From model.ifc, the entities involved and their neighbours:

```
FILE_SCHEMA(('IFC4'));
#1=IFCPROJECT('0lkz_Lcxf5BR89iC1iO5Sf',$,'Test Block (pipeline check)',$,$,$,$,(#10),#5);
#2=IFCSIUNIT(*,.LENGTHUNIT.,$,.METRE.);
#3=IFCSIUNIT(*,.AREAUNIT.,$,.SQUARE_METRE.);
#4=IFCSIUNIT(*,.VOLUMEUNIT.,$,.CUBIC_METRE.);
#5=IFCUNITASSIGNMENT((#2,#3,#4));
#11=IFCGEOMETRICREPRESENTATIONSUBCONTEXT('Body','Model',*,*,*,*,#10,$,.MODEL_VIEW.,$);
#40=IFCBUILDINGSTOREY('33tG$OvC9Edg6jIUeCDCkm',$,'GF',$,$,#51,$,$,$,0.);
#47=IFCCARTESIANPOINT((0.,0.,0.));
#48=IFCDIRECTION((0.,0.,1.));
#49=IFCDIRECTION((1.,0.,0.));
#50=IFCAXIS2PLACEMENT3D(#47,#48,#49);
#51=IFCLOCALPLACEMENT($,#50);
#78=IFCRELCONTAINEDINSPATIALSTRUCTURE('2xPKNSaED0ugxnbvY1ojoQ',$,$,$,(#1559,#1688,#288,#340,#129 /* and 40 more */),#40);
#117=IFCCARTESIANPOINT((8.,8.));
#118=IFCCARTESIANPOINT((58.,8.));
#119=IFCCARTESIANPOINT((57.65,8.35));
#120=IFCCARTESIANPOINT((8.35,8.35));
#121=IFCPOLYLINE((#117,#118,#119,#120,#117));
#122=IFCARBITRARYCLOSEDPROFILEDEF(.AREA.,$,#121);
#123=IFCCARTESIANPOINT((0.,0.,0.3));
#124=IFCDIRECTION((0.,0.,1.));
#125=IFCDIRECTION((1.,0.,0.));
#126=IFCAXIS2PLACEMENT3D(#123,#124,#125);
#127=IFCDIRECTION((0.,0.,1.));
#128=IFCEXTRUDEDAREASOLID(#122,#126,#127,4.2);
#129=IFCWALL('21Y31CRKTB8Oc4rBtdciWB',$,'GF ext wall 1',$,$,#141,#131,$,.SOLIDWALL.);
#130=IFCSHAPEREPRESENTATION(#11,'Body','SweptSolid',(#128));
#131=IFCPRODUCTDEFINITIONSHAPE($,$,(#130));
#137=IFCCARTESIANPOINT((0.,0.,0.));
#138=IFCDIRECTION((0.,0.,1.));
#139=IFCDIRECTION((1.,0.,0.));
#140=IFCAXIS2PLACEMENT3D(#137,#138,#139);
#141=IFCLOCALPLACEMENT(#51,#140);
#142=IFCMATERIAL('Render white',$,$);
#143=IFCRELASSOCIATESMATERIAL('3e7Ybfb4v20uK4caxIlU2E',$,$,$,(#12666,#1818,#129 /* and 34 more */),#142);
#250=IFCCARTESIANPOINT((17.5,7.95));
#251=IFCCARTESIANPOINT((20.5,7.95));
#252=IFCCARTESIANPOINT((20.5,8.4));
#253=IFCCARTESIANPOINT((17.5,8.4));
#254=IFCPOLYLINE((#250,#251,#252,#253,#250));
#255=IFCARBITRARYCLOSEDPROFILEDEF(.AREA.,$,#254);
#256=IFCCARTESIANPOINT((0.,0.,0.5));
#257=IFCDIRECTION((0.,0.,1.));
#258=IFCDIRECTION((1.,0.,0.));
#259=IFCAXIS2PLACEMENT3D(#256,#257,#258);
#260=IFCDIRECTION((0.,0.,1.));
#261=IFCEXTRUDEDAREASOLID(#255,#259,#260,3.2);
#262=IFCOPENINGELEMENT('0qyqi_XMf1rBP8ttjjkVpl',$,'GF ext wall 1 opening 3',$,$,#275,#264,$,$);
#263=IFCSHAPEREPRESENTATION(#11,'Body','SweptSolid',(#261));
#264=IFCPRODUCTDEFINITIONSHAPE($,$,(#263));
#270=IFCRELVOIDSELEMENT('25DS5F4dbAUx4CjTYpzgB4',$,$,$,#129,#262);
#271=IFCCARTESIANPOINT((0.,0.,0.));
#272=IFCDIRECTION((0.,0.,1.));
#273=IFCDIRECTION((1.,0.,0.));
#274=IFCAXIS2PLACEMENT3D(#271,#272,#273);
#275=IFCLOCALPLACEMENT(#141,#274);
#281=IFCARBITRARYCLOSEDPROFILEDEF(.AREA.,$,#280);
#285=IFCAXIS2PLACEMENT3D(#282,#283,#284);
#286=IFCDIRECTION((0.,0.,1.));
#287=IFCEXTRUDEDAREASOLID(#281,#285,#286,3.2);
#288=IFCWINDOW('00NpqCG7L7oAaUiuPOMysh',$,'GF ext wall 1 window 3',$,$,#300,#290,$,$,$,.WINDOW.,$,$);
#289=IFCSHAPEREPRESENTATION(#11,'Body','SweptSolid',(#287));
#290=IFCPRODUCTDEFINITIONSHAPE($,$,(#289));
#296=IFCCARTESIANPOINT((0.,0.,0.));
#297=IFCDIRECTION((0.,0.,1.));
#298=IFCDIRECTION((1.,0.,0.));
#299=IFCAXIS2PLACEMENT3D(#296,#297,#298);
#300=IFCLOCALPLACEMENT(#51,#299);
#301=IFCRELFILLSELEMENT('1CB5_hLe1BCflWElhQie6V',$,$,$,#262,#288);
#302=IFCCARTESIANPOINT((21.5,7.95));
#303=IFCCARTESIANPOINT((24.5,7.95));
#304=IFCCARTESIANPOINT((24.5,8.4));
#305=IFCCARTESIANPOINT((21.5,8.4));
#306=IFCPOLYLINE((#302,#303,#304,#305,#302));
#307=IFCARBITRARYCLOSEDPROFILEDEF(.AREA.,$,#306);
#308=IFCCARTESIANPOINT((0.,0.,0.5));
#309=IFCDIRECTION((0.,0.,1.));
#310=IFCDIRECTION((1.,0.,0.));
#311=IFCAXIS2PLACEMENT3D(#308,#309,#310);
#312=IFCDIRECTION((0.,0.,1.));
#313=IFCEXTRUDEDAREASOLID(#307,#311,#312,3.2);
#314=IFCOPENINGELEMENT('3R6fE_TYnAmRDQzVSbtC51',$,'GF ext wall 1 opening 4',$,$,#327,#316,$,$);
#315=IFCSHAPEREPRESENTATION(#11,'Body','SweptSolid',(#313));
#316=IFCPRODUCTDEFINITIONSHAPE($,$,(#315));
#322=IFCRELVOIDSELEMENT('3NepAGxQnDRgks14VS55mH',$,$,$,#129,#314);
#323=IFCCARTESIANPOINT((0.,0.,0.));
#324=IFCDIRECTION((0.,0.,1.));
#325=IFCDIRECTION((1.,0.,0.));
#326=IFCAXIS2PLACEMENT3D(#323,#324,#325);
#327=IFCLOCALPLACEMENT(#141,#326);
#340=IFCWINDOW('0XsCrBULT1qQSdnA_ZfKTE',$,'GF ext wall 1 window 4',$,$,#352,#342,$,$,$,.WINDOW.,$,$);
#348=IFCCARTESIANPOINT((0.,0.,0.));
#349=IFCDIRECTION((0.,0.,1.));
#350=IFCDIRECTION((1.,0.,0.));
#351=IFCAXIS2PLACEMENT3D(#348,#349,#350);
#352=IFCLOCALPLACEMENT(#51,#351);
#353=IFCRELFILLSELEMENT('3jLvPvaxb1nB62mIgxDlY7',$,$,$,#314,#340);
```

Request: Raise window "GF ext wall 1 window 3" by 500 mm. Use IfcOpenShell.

```python
import numpy as np
import ifcopenshell
import ifcopenshell.api.geometry
import ifcopenshell.util.placement
import ifcopenshell.util.unit

model = ifcopenshell.open("model.ifc")
unit_scale = ifcopenshell.util.unit.calculate_unit_scale(model)

window = model.by_guid("00NpqCG7L7oAaUiuPOMysh")
opening = window.FillsVoids[0].RelatingOpeningElement
dz = 0.5 / unit_scale

shift = np.array([0.0, 0.0, dz])
# The window is not placed relative to its opening, so move both.
for product in (opening, window):
    matrix = ifcopenshell.util.placement.get_local_placement(product.ObjectPlacement)
    matrix[:3, 3] += shift
    ifcopenshell.api.geometry.edit_object_placement(model, product=product, matrix=matrix, is_si=False)

print(f"moved by {dz * unit_scale:+.3f} m")

model.write("model_updated.ifc")
```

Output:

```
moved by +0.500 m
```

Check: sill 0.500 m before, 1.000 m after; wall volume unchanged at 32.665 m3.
